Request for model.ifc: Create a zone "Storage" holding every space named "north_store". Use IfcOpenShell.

First a look at what the model holds.

```python
import ifcopenshell

model = ifcopenshell.open("model.ifc")
print(model.schema)
seen = {}
for space in model.by_type("IfcSpace"):
    seen[space.Name] = seen.get(space.Name, 0) + 1
for name, count in sorted(seen.items(), key=str):
    print(count, "x", name)
print("zones:", [z.Name for z in model.by_type("IfcZone")][:20])
```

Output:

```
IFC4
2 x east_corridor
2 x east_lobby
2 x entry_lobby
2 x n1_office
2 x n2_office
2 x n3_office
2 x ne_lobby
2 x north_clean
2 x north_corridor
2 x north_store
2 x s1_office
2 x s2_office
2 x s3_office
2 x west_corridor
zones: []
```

```python
import ifcopenshell
import ifcopenshell.api.group
import ifcopenshell.api.root

model = ifcopenshell.open("model.ifc")

names = {"north_store"}
spaces = [s for s in model.by_type("IfcSpace") if s.Name in names]

zone = ifcopenshell.api.root.create_entity(model, ifc_class="IfcZone", name="Storage")
ifcopenshell.api.group.assign_group(model, products=spaces, group=zone)
print(len(spaces), "spaces in", zone.Name)

model.write("model_updated.ifc")
```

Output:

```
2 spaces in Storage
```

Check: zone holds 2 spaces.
